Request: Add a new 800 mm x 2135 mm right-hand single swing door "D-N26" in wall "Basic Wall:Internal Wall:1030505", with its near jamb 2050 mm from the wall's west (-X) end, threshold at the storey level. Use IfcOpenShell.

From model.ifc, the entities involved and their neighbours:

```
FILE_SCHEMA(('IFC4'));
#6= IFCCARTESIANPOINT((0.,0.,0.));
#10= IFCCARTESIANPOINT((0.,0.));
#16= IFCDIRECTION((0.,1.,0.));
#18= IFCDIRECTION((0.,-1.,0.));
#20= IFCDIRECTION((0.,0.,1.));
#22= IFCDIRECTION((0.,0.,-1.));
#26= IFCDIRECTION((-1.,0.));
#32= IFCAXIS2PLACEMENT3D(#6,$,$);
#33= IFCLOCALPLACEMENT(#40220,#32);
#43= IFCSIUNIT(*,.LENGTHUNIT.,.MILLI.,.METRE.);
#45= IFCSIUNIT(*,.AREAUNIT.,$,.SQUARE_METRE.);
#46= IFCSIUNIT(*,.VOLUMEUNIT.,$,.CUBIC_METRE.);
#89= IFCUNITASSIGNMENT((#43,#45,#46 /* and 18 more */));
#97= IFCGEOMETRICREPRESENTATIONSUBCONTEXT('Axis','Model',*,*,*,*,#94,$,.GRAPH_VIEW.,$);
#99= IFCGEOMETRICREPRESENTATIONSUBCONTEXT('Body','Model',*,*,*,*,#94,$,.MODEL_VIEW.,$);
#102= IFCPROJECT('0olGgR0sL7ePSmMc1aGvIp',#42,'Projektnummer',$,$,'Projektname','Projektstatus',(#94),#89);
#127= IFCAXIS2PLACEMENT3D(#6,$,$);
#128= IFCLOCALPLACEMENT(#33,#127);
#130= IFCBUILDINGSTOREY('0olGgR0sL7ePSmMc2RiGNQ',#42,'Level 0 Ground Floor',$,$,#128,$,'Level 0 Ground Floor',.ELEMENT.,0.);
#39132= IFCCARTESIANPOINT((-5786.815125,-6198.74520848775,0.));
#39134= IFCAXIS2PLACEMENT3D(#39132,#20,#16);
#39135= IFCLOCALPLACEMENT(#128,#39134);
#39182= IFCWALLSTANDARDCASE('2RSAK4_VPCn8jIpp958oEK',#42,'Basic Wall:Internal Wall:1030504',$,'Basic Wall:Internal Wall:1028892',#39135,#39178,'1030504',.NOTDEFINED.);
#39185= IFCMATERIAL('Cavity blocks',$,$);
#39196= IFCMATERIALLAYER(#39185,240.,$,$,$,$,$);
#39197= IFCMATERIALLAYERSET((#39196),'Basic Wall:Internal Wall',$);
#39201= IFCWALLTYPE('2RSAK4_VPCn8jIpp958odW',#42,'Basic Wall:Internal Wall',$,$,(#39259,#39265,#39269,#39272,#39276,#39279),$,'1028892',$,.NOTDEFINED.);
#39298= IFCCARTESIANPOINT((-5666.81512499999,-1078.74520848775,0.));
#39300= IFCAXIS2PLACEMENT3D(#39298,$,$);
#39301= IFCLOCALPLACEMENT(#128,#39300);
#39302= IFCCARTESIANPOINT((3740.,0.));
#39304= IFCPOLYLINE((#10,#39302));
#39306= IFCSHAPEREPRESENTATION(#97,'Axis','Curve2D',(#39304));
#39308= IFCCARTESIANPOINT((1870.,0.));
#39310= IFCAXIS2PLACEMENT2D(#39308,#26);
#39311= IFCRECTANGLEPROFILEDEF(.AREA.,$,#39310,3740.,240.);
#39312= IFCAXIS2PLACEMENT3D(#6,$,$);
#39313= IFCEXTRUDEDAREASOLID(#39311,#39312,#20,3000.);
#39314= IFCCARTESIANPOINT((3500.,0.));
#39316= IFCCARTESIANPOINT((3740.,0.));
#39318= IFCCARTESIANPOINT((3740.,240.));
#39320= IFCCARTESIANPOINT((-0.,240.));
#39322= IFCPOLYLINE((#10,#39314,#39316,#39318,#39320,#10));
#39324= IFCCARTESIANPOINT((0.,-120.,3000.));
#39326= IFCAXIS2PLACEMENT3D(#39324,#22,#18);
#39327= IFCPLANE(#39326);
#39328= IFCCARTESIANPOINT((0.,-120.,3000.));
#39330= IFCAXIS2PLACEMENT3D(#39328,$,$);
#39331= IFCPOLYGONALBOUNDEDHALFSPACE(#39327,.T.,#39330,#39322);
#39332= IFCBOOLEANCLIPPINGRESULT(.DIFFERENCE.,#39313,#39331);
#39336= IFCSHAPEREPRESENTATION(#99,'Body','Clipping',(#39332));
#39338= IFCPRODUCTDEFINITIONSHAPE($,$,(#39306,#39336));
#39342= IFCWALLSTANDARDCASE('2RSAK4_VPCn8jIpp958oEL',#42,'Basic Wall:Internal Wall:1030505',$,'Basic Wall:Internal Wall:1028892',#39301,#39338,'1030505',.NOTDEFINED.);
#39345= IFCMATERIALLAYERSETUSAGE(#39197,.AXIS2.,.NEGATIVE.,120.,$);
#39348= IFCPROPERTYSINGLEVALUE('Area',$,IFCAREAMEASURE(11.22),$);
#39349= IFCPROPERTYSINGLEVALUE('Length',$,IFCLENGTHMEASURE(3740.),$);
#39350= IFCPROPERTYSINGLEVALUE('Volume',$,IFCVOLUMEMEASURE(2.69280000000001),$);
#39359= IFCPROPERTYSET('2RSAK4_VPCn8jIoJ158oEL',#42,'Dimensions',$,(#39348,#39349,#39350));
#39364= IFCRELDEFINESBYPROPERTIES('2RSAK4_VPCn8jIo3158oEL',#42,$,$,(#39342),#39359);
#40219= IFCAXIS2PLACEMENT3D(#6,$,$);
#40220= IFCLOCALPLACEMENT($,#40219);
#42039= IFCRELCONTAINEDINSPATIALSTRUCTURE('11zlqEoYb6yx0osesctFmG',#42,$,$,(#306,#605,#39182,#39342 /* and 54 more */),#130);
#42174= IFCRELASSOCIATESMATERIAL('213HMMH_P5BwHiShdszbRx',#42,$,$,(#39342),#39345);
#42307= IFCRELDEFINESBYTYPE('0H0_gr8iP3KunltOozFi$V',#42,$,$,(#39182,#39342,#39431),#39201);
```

```python
import numpy as np
import ifcopenshell
import ifcopenshell.api.feature
import ifcopenshell.api.geometry
import ifcopenshell.api.pset
import ifcopenshell.api.root
import ifcopenshell.api.spatial
import ifcopenshell.geom
import ifcopenshell.util.element
import ifcopenshell.util.placement
import ifcopenshell.util.representation
import ifcopenshell.util.shape
import ifcopenshell.util.unit

model = ifcopenshell.open("model.ifc")
unit_scale = ifcopenshell.util.unit.calculate_unit_scale(model)
area_scale = ifcopenshell.util.unit.calculate_unit_scale(model, "AREAUNIT")
volume_scale = ifcopenshell.util.unit.calculate_unit_scale(model, "VOLUMEUNIT")
settings = ifcopenshell.geom.settings()


def volume(element):
    """Net volume in cubic metres, openings subtracted."""
    shape = ifcopenshell.geom.create_shape(settings, element)
    return ifcopenshell.util.shape.get_volume(shape.geometry)


wall = model.by_guid("2RSAK4_VPCn8jIpp958oEL")
storey = ifcopenshell.util.element.get_container(wall, ifc_class="IfcBuildingStorey")
context = ifcopenshell.util.representation.get_context(model, "Model", "Body", "MODEL_VIEW")
before = volume(wall)

width, height, from_end, sill = 0.8, 2.135, 2.05, 0.0  # metres

# The wall runs along its own X axis, and the end named is its -X end.
wall_shape = ifcopenshell.geom.create_shape(settings, wall)
x, y, z = ifcopenshell.util.shape.get_vertices(wall_shape.geometry).T
start = x.min() + from_end
face, thickness = float(y.min()), float(y.max() - y.min())
wall_matrix = ifcopenshell.util.placement.get_local_placement(wall.ObjectPlacement)
level = ifcopenshell.util.placement.get_local_placement(storey.ObjectPlacement)[2, 3]


def in_wall(x, y):
    """Placement at x, y metres in the wall's axes, at sill height."""
    matrix = wall_matrix.copy()
    matrix[:, 3] = wall_matrix @ np.array([x / unit_scale, y / unit_scale, 0.0, 1.0])
    matrix[2, 3] = level + sill / unit_scale
    return matrix


# Opening: a box that overshoots both wall faces by 50 mm.
opening = ifcopenshell.api.root.create_entity(model, ifc_class="IfcOpeningElement", predefined_type="OPENING")
box = ifcopenshell.api.geometry.add_wall_representation(
    model, context=context, length=width, height=height, thickness=thickness + 0.1
)
ifcopenshell.api.geometry.assign_representation(model, product=opening, representation=box)
ifcopenshell.api.geometry.edit_object_placement(model, product=opening, matrix=in_wall(start, face - 0.05), is_si=False)
ifcopenshell.api.feature.add_feature(model, feature=opening, element=wall)

door = ifcopenshell.api.root.create_entity(model, ifc_class="IfcDoor", name="D-N26", predefined_type="DOOR")
door.OverallWidth, door.OverallHeight = width / unit_scale, height / unit_scale
door.OperationType = "SINGLE_SWING_RIGHT"
body = ifcopenshell.api.geometry.add_door_representation(
    model,
    context=context,
    overall_width=door.OverallWidth,
    overall_height=door.OverallHeight,
    operation_type="SINGLE_SWING_RIGHT",
    lining_properties={"LiningDepth": thickness / unit_scale, "ThresholdDepth": thickness / unit_scale},
)
ifcopenshell.api.geometry.assign_representation(model, product=door, representation=body)
ifcopenshell.api.spatial.assign_container(model, products=[door], relating_structure=storey)
ifcopenshell.api.feature.add_filling(model, opening=opening, element=door)

# The lining spans the wall, so the door starts at the wall face.
ifcopenshell.api.geometry.edit_object_placement(model, product=door, matrix=in_wall(start, face), is_si=False)

after = volume(wall)

# Update the wall's stored quantities.
pset = model.by_id(ifcopenshell.util.element.get_pset(wall, "Dimensions", should_inherit=False)["id"])
ifcopenshell.api.pset.edit_pset(model, pset=pset, properties={
    "Area": model.create_entity("IfcAreaMeasure", after / thickness / area_scale),
    "Volume": model.create_entity("IfcVolumeMeasure", after / volume_scale),
})

print(f"wall volume {before:.3f} -> {after:.3f} m3")

model.write("model-out.ifc")
```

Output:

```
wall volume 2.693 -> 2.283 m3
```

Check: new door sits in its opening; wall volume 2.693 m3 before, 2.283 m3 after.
